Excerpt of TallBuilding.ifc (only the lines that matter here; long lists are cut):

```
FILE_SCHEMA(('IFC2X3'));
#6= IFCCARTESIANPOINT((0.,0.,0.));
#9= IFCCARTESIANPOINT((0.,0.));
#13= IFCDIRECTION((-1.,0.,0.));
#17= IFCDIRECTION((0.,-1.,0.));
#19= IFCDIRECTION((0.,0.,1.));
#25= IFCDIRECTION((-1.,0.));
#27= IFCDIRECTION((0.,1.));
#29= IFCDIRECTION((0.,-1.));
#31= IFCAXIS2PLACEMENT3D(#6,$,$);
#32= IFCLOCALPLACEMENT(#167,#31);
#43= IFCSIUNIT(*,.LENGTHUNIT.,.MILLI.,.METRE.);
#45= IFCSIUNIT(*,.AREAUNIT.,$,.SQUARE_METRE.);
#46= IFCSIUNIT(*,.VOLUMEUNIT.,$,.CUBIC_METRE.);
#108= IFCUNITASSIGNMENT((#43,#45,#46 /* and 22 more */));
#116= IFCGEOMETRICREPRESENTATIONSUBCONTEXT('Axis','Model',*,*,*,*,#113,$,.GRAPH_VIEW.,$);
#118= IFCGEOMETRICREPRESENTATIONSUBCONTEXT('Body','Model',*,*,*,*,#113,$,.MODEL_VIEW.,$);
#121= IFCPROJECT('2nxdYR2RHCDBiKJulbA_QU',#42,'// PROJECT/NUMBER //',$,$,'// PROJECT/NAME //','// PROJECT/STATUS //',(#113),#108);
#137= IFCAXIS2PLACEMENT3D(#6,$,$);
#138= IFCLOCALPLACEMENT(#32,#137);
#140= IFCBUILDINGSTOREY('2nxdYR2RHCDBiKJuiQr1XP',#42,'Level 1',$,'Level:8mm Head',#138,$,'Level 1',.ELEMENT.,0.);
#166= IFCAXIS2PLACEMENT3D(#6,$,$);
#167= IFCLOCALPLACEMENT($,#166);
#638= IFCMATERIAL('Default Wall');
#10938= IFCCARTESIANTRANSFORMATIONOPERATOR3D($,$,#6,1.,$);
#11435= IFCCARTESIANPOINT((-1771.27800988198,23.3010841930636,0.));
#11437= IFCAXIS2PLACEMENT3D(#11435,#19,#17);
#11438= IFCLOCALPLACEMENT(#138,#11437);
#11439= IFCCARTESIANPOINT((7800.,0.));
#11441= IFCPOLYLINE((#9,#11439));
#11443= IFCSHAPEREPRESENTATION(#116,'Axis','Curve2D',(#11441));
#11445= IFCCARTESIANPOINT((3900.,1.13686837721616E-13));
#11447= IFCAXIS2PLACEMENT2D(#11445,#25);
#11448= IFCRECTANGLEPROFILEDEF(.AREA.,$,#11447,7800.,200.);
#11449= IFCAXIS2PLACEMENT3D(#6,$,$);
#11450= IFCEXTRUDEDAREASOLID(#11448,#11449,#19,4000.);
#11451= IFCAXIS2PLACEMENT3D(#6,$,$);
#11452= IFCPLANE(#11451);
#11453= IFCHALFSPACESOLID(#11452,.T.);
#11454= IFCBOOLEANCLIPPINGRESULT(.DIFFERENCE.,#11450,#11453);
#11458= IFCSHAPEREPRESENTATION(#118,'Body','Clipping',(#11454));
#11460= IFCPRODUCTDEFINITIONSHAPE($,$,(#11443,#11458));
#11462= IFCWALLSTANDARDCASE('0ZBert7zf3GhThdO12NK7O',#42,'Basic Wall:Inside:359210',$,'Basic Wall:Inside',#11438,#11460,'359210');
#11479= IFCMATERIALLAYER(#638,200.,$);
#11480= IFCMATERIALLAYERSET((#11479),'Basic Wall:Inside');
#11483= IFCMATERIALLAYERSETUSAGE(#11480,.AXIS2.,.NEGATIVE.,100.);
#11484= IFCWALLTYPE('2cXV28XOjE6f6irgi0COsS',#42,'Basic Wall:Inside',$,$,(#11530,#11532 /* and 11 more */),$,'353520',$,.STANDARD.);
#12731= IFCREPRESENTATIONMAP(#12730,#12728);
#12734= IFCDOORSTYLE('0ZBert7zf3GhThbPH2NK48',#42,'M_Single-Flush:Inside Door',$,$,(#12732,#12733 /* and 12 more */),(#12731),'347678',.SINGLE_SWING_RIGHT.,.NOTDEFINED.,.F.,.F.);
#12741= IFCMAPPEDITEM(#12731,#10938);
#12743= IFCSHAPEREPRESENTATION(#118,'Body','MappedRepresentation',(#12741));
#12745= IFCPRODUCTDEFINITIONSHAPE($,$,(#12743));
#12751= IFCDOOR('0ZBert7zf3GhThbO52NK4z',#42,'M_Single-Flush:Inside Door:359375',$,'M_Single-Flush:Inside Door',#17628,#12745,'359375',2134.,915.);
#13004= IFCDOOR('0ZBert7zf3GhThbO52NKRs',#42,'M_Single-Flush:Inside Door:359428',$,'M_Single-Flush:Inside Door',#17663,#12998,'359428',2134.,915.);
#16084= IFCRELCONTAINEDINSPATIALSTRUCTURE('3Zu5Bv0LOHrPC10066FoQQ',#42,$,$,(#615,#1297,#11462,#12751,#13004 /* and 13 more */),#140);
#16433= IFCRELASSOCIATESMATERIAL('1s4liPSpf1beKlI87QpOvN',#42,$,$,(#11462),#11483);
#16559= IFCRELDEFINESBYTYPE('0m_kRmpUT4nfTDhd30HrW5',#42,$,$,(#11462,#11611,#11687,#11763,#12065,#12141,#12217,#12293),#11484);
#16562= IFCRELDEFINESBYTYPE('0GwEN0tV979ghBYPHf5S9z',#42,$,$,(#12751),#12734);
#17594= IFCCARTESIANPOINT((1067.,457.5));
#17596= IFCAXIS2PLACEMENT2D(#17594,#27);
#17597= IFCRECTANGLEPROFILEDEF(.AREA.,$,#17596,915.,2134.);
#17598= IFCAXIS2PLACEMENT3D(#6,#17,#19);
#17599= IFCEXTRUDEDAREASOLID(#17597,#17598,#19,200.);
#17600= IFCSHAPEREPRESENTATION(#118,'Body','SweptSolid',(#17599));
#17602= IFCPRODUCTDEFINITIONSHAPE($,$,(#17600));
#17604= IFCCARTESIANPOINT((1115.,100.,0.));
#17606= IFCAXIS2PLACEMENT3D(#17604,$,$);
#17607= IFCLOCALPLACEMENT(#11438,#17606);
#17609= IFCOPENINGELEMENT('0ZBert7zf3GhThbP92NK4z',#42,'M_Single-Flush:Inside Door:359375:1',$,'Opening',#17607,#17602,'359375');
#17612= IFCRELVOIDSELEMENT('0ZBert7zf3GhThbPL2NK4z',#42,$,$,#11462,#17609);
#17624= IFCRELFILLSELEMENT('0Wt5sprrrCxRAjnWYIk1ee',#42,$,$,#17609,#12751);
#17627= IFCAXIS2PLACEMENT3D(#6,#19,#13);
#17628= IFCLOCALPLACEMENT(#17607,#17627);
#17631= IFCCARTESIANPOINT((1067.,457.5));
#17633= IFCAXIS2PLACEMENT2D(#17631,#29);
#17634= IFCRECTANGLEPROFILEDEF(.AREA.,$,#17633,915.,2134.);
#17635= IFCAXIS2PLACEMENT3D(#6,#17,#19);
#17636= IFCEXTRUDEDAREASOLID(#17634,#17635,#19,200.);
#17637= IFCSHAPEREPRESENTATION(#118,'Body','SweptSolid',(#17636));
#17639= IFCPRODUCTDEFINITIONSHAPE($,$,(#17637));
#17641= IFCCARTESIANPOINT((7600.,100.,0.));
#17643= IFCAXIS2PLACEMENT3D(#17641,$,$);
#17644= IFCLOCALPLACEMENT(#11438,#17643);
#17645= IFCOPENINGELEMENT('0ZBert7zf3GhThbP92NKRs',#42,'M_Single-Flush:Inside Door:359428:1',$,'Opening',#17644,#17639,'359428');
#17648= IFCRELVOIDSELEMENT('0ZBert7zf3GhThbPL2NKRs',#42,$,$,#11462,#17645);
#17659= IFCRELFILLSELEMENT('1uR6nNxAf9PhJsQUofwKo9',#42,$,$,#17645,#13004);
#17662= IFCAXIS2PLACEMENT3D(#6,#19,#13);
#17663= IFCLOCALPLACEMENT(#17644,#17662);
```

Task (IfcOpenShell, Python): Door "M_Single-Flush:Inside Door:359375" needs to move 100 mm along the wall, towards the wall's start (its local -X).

```python
import ifcopenshell
import ifcopenshell.api.geometry
import ifcopenshell.util.placement
import ifcopenshell.util.unit

model = ifcopenshell.open("TallBuilding.ifc")
unit_scale = ifcopenshell.util.unit.calculate_unit_scale(model)

door = model.by_guid("0ZBert7zf3GhThbO52NK4z")
opening = door.FillsVoids[0].RelatingOpeningElement
wall = opening.VoidsElements[0].RelatingBuildingElement

wall_matrix = ifcopenshell.util.placement.get_local_placement(wall.ObjectPlacement)
shift = wall_matrix[:3, 0] * -0.1 / unit_scale
before = ifcopenshell.util.placement.get_local_placement(door.ObjectPlacement)[:3, 3].copy()

# The door is placed relative to its opening, so it follows when the opening moves.
matrix = ifcopenshell.util.placement.get_local_placement(opening.ObjectPlacement)
matrix[:3, 3] += shift
ifcopenshell.api.geometry.edit_object_placement(
    model, product=opening, matrix=matrix, is_si=False, should_transform_children=True
)

after = ifcopenshell.util.placement.get_local_placement(door.ObjectPlacement)[:3, 3]
print("door moved by", (after - before).round(3) + 0.0)

model.write("TallBuilding_rev.ifc")
```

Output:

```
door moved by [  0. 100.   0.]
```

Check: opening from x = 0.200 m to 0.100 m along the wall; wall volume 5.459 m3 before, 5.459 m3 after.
